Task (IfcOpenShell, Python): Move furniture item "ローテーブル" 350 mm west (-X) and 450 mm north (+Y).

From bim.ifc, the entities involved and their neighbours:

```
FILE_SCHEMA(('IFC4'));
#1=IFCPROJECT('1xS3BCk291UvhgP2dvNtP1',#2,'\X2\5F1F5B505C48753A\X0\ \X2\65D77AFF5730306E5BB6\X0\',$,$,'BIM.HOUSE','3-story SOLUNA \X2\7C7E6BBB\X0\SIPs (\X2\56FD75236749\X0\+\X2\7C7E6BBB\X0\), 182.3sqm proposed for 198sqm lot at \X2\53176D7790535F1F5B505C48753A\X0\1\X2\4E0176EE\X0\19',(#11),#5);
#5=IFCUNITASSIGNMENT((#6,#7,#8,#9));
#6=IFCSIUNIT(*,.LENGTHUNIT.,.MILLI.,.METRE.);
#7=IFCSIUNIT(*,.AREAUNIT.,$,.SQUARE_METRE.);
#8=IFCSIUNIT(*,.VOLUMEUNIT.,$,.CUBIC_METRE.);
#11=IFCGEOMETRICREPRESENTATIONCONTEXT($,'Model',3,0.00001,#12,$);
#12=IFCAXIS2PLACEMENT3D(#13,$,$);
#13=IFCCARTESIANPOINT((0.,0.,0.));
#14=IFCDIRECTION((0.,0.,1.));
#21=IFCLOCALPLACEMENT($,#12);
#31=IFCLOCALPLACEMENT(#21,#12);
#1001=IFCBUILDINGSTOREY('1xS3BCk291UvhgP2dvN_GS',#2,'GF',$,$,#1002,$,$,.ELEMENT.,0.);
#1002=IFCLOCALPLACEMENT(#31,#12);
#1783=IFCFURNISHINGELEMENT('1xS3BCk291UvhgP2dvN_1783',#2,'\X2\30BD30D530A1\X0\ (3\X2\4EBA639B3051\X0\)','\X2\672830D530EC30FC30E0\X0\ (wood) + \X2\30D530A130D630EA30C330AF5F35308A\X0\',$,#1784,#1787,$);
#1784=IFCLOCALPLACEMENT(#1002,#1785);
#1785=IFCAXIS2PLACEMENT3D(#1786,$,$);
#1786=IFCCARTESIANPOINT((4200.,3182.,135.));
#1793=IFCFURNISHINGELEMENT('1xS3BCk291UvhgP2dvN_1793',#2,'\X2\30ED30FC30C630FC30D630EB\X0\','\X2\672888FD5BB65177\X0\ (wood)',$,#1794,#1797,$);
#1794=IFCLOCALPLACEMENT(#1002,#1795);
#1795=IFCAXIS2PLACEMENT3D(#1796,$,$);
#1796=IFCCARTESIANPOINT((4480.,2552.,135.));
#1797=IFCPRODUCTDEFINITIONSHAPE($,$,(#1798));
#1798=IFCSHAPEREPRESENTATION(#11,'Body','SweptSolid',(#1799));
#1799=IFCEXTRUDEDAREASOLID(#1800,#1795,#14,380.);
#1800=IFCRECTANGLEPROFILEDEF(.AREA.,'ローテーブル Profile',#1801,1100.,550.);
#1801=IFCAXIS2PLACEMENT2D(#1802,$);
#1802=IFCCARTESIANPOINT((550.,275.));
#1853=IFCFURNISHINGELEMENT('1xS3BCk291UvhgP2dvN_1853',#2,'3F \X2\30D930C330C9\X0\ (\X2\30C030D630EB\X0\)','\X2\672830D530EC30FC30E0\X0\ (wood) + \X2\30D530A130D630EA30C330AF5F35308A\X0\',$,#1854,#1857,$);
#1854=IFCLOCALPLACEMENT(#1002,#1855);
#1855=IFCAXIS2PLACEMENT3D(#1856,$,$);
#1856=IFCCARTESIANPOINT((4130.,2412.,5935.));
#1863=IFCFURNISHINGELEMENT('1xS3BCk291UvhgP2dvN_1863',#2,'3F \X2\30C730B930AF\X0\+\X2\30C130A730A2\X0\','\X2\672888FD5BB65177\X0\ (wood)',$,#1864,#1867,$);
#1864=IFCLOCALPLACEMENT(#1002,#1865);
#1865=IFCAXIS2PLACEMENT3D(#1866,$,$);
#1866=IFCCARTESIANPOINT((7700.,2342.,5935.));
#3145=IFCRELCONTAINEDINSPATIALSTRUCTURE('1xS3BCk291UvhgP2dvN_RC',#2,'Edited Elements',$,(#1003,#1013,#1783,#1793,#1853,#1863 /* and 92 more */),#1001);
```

```python
import ifcopenshell
import ifcopenshell.api.geometry
import ifcopenshell.util.placement

model = ifcopenshell.open("bim.ifc")

item = model.by_guid("1xS3BCk291UvhgP2dvN_1793")
matrix = ifcopenshell.util.placement.get_local_placement(item.ObjectPlacement)
matrix[0, 3] -= 350.0
matrix[1, 3] += 450.0
ifcopenshell.api.geometry.edit_object_placement(model, product=item, matrix=matrix, is_si=False)

print(ifcopenshell.util.placement.get_local_placement(item.ObjectPlacement).round(3) + 0.0)

model.write("bim-out.ifc")
```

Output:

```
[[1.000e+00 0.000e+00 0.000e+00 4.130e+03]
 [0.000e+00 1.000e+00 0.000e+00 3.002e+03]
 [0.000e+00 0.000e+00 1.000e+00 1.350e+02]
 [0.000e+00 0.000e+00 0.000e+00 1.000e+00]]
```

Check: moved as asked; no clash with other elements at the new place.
